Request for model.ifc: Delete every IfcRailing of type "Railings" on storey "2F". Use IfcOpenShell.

First a look at what the model holds.

```python
import ifcopenshell
import ifcopenshell.util.element

model = ifcopenshell.open("model.ifc")
print(model.schema)
storey = next(s for s in model.by_type("IfcBuildingStorey") if s.Name == "2F")
railings = [e for e in ifcopenshell.util.element.get_decomposition(storey) if e.is_a("IfcRailing")]
seen = {}
for e in railings:
    element_type = ifcopenshell.util.element.get_type(e)
    name = element_type.Name if element_type not in (None, e) else None
    seen[name] = seen.get(name, 0) + 1
for name, count in sorted(seen.items(), key=str):
    print(count, "x", name)
```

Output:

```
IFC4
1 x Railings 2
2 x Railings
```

```python
import ifcopenshell
import ifcopenshell.api.root
import ifcopenshell.util.element

model = ifcopenshell.open("model.ifc")

storey = next(s for s in model.by_type("IfcBuildingStorey") if s.Name == "2F")
railings = [e for e in ifcopenshell.util.element.get_decomposition(storey) if e.is_a("IfcRailing")]
targets = [e for e in railings if (t := ifcopenshell.util.element.get_type(e)) not in (None, e) and t.Name == "Railings"]

for e in targets:
    ifcopenshell.api.root.remove_product(model, product=e)
print(len(targets), "removed")

model.write("model_updated.ifc")
```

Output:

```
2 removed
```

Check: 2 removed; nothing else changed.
